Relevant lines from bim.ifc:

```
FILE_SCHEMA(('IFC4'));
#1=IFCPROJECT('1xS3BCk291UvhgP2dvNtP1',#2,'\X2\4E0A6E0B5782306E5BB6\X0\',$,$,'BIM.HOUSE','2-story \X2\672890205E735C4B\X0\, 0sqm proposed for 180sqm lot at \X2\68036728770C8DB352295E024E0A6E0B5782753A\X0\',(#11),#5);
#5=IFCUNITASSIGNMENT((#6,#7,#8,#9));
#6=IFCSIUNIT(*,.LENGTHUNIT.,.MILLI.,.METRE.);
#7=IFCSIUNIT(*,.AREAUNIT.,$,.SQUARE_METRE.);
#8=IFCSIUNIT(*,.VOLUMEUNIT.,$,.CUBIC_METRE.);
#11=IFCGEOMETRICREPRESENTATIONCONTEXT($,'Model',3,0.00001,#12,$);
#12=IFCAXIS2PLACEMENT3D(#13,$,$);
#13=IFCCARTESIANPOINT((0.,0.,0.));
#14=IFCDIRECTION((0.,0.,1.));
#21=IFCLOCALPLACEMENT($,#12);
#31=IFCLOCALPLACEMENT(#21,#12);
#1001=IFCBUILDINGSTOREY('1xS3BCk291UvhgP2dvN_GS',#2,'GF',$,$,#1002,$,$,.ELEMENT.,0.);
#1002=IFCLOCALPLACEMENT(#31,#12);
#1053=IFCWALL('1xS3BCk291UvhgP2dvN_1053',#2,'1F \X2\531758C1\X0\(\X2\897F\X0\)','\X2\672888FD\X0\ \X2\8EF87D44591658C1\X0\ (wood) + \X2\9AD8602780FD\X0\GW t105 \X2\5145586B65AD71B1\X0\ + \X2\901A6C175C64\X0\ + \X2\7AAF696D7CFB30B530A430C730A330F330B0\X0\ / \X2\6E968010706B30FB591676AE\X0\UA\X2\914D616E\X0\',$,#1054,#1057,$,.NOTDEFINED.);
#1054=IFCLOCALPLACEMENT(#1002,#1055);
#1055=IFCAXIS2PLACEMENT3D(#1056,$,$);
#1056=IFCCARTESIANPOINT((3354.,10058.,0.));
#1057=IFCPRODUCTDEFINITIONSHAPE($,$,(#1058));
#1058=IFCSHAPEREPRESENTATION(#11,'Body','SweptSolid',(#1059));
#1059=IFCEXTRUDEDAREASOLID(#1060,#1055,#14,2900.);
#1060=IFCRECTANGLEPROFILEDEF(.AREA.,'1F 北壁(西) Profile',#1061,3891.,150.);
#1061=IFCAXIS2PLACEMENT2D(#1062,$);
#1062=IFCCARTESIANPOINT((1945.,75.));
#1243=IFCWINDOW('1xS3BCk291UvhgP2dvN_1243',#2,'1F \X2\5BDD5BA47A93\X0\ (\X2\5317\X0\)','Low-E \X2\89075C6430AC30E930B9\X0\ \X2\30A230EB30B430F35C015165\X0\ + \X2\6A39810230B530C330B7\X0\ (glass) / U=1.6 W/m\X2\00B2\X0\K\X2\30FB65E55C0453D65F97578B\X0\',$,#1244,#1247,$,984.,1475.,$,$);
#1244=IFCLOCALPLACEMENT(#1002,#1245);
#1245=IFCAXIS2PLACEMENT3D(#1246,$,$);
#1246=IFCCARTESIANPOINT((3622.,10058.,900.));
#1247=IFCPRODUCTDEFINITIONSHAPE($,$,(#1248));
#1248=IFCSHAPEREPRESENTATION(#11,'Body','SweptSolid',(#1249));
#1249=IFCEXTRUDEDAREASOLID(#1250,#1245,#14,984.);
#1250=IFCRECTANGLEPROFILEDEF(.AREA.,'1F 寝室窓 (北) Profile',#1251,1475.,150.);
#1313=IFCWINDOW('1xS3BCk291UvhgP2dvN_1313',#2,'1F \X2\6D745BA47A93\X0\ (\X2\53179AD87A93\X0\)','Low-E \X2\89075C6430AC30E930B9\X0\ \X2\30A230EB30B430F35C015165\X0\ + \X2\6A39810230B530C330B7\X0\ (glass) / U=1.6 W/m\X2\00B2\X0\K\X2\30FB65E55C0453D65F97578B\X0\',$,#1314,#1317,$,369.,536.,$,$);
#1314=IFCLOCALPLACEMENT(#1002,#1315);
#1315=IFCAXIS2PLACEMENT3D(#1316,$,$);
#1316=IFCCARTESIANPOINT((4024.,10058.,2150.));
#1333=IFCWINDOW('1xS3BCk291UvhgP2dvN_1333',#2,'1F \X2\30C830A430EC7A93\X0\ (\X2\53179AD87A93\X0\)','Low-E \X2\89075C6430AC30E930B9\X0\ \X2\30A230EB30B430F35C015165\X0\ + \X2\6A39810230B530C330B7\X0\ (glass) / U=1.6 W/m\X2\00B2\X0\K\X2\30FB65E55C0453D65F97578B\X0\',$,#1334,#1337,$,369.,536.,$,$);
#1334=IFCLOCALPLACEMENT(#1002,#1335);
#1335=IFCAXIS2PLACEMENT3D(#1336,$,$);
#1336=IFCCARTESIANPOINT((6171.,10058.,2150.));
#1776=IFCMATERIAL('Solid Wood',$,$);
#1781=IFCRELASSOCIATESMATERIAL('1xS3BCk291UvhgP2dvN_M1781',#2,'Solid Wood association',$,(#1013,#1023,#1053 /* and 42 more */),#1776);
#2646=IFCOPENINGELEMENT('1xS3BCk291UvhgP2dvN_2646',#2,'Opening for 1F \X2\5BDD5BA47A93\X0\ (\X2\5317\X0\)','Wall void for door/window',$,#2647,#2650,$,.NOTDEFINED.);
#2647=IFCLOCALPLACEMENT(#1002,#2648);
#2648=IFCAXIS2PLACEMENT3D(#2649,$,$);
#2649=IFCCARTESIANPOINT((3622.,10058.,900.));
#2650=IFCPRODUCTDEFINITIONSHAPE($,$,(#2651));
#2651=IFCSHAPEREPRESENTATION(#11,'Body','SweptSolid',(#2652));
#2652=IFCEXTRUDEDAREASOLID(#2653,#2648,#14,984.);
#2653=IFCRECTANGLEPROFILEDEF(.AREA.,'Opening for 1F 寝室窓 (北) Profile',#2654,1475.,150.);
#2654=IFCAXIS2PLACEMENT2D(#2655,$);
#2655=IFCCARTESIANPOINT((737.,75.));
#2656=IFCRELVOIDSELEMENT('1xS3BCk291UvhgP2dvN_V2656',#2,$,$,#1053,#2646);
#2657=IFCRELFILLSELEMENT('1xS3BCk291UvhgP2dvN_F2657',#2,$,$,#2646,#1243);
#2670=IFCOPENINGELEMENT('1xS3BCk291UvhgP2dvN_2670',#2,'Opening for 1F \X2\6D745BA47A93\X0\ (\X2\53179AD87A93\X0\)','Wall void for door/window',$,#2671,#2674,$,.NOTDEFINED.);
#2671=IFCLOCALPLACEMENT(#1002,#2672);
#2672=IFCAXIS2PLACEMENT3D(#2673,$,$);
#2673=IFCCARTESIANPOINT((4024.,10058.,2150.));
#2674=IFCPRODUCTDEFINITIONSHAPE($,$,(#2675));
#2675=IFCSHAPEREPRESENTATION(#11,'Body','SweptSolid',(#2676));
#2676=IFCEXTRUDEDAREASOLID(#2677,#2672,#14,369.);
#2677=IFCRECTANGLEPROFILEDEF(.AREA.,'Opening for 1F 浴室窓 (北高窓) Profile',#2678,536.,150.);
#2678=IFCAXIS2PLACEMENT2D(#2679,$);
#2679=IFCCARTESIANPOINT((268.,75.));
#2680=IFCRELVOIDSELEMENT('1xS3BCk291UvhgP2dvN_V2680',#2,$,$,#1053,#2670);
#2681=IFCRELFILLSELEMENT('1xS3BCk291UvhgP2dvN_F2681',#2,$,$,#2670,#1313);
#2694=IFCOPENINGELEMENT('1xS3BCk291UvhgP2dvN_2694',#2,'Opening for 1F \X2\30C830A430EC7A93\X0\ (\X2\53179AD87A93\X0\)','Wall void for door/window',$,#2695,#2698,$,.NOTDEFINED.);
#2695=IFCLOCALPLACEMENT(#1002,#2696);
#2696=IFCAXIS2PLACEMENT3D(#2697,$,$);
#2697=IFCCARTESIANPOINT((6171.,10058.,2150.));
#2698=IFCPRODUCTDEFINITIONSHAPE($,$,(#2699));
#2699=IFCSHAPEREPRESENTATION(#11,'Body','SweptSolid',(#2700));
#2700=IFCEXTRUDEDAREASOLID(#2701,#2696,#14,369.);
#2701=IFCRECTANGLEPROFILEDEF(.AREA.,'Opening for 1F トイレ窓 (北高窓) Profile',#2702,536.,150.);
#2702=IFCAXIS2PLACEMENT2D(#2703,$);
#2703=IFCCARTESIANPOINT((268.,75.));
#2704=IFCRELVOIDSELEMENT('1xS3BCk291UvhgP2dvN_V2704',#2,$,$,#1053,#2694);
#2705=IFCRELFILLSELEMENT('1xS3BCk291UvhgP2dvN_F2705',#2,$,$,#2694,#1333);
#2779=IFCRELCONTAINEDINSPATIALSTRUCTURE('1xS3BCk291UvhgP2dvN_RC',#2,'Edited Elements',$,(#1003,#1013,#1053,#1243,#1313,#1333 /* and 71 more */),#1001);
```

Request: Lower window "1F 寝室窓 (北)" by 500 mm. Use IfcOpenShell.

```python
import numpy as np
import ifcopenshell
import ifcopenshell.api.geometry
import ifcopenshell.util.placement
import ifcopenshell.util.unit

model = ifcopenshell.open("bim.ifc")
unit_scale = ifcopenshell.util.unit.calculate_unit_scale(model)

window = model.by_id(1243)
opening = window.FillsVoids[0].RelatingOpeningElement
dz = -500.0

shift = np.array([0.0, 0.0, dz])
# The window is not placed relative to its opening, so move both.
for product in (opening, window):
    matrix = ifcopenshell.util.placement.get_local_placement(product.ObjectPlacement)
    matrix[:3, 3] += shift
    ifcopenshell.api.geometry.edit_object_placement(model, product=product, matrix=matrix, is_si=False)

print(f"moved by {dz * unit_scale:+.3f} m")

model.write("bim_updated.ifc")
```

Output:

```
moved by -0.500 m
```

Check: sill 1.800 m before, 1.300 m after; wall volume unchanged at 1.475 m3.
